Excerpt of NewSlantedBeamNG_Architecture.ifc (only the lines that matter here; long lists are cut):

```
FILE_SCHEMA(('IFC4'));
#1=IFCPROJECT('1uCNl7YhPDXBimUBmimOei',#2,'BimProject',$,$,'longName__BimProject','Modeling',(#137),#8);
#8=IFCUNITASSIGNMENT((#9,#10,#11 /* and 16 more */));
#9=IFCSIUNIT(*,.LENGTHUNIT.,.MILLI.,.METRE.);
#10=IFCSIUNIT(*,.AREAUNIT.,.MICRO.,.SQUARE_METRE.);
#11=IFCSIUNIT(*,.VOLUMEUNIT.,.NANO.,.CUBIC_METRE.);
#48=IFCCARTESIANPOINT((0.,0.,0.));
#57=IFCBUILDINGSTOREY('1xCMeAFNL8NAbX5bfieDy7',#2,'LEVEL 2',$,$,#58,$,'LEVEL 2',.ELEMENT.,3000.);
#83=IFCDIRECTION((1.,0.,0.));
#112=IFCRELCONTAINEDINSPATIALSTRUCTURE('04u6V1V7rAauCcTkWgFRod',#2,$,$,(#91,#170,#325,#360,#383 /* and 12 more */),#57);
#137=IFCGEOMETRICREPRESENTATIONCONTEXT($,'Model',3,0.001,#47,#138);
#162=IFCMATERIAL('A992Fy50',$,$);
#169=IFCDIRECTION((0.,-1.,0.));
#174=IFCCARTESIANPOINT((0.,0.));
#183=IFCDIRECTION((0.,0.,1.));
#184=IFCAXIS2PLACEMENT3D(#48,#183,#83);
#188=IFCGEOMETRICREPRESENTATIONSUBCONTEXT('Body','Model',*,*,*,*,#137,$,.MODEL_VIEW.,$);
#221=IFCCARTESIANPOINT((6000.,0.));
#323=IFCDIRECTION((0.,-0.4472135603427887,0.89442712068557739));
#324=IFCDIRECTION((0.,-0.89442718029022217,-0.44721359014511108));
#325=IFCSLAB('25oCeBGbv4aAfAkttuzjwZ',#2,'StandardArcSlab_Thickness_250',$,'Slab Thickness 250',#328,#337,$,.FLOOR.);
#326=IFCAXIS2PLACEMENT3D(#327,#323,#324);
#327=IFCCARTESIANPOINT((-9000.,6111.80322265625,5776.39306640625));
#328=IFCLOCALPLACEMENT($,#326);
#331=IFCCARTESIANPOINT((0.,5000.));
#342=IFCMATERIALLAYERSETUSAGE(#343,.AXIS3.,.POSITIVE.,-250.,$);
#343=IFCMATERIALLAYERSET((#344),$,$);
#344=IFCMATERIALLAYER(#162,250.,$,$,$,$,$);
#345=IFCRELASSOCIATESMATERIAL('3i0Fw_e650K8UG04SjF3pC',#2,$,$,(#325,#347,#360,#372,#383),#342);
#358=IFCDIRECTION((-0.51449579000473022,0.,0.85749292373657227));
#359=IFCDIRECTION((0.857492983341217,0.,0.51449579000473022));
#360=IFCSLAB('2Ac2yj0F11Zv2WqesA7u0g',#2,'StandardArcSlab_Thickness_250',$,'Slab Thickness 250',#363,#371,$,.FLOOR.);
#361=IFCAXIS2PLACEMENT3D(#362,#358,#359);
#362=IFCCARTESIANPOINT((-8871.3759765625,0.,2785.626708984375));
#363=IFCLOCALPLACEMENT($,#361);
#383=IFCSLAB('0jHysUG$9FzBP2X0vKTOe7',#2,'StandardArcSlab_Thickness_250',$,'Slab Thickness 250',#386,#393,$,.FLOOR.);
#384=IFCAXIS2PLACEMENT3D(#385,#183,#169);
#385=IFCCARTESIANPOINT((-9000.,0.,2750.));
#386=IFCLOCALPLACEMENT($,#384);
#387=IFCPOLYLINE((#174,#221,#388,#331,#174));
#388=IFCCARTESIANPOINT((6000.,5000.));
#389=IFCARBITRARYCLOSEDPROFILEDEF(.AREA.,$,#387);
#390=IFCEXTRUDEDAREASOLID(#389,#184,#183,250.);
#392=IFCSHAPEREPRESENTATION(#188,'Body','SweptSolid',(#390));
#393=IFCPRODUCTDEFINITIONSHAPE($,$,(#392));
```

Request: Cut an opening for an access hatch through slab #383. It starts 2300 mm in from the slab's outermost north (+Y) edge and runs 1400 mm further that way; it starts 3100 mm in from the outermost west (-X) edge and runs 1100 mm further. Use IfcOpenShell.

```python
import numpy as np
import ifcopenshell
import ifcopenshell.api.feature
import ifcopenshell.api.geometry
import ifcopenshell.api.root
import ifcopenshell.geom
import ifcopenshell.util.placement
import ifcopenshell.util.representation
import ifcopenshell.util.shape
import ifcopenshell.util.unit

model = ifcopenshell.open("NewSlantedBeamNG_Architecture.ifc")
unit_scale = ifcopenshell.util.unit.calculate_unit_scale(model)
settings = ifcopenshell.geom.settings()


def volume(element):
    """Net volume in cubic metres, openings subtracted."""
    shape = ifcopenshell.geom.create_shape(settings, element)
    return ifcopenshell.util.shape.get_volume(shape.geometry)


slab = model.by_id(383)
before = volume(slab)

# Extent in the slab's own axes, in metres. The edges named are its -X and -Y sides.
slab_shape = ifcopenshell.geom.create_shape(settings, slab)
vertices = ifcopenshell.util.shape.get_vertices(slab_shape.geometry)
x_min, y_min, bottom = vertices.min(axis=0)
top = vertices[:, 2].max()

opening = ifcopenshell.api.root.create_entity(model, ifc_class="IfcOpeningElement", name="Access hatch opening", predefined_type="OPENING")
context = ifcopenshell.util.representation.get_context(model, "Model", "Body", "MODEL_VIEW")
width, depth = 1.4, 1.1
outline = [(0.0, 0.0), (width, 0.0), (width, depth), (0.0, depth), (0.0, 0.0)]
# Overshoot both faces by 50 mm so the cut is clean.
shape = ifcopenshell.api.geometry.add_slab_representation(
    model, context=context, depth=top - bottom + 0.1, polyline=outline
)
ifcopenshell.api.geometry.assign_representation(model, product=opening, representation=shape)

matrix = ifcopenshell.util.placement.get_local_placement(slab.ObjectPlacement)
matrix[:, 3] = matrix @ np.append(np.array([x_min + 2.3, y_min + 3.1, bottom - 0.05]) / unit_scale, 1.0)
ifcopenshell.api.geometry.edit_object_placement(model, product=opening, matrix=matrix, is_si=False)
ifcopenshell.api.feature.add_feature(model, feature=opening, element=slab)

after = volume(slab)

print(f"slab volume {before:.3f} -> {after:.3f} m3")

model.write("NewSlantedBeamNG_Architecture_v2.ifc")
```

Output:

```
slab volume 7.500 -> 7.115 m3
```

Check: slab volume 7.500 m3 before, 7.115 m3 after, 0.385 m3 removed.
